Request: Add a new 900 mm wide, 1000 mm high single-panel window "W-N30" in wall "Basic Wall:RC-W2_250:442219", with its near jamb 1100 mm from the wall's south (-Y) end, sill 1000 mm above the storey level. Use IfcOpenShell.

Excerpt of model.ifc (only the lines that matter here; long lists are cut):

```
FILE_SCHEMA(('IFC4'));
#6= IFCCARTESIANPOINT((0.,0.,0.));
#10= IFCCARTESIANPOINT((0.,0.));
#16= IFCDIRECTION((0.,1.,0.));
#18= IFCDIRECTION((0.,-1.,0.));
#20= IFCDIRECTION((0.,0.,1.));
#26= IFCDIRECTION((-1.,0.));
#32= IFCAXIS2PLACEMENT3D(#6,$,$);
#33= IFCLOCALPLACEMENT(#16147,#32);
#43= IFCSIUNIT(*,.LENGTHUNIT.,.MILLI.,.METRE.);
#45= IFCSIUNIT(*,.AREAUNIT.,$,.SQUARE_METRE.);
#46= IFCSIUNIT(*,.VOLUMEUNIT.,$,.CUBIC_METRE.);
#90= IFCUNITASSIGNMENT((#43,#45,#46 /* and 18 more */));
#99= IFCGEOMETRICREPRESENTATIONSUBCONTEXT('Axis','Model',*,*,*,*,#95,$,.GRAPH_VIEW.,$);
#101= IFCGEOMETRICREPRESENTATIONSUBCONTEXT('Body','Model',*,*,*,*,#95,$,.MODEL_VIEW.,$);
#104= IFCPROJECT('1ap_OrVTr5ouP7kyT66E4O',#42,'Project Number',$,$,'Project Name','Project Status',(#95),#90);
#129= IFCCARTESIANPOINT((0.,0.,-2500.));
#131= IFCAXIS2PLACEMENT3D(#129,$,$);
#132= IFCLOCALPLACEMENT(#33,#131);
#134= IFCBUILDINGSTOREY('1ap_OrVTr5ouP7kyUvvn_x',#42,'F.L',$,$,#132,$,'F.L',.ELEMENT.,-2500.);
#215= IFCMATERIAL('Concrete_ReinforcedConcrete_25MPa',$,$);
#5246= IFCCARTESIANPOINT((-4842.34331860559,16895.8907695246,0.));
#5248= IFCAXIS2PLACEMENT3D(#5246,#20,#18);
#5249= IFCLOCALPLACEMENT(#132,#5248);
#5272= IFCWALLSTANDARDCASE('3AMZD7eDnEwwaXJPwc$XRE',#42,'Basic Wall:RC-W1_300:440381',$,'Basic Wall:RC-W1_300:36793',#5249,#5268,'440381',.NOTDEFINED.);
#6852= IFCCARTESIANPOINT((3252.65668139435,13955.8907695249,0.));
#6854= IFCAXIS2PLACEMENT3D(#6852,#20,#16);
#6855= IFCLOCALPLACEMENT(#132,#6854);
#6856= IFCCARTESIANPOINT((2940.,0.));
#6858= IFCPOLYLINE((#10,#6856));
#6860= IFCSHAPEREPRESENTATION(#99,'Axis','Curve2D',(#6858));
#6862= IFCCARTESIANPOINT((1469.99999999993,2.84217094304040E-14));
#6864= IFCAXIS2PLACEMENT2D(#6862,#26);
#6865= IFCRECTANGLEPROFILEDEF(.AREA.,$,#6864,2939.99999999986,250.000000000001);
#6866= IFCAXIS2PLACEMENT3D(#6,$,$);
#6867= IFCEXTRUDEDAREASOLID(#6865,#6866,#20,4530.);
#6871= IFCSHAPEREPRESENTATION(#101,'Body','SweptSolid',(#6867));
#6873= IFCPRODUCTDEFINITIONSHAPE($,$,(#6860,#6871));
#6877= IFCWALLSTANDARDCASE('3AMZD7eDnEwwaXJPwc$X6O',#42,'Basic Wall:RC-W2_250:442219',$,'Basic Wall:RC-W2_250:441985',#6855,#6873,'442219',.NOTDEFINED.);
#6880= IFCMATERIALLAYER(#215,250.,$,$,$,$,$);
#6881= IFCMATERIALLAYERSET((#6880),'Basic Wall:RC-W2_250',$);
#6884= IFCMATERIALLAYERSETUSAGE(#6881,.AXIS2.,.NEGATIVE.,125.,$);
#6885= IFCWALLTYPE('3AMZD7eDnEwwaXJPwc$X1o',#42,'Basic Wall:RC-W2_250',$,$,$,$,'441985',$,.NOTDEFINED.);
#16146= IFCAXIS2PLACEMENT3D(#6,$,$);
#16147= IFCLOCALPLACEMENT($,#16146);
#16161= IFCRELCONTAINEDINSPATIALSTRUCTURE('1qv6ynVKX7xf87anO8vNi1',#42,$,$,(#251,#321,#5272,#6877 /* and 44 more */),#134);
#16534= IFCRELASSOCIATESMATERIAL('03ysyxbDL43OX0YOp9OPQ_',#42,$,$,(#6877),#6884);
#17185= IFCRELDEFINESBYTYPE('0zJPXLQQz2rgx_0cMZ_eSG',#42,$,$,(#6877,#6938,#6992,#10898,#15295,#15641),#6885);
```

```python
import numpy as np
import ifcopenshell
import ifcopenshell.api.feature
import ifcopenshell.api.geometry
import ifcopenshell.api.root
import ifcopenshell.api.spatial
import ifcopenshell.geom
import ifcopenshell.util.element
import ifcopenshell.util.placement
import ifcopenshell.util.representation
import ifcopenshell.util.shape
import ifcopenshell.util.unit

model = ifcopenshell.open("model.ifc")
unit_scale = ifcopenshell.util.unit.calculate_unit_scale(model)
settings = ifcopenshell.geom.settings()


def volume(element):
    """Net volume in cubic metres, openings subtracted."""
    shape = ifcopenshell.geom.create_shape(settings, element)
    return ifcopenshell.util.shape.get_volume(shape.geometry)


wall = model.by_guid("3AMZD7eDnEwwaXJPwc$X6O")
storey = ifcopenshell.util.element.get_container(wall, ifc_class="IfcBuildingStorey")
context = ifcopenshell.util.representation.get_context(model, "Model", "Body", "MODEL_VIEW")
before = volume(wall)

width, height, from_end, sill = 0.9, 1, 1.1, 1  # metres

# The wall runs along its own X axis, and the end named is its -X end.
wall_shape = ifcopenshell.geom.create_shape(settings, wall)
x, y, z = ifcopenshell.util.shape.get_vertices(wall_shape.geometry).T
start = x.min() + from_end
face, thickness = float(y.min()), float(y.max() - y.min())
wall_matrix = ifcopenshell.util.placement.get_local_placement(wall.ObjectPlacement)
level = ifcopenshell.util.placement.get_local_placement(storey.ObjectPlacement)[2, 3]


def in_wall(x, y):
    """Placement at x, y metres in the wall's axes, at sill height."""
    matrix = wall_matrix.copy()
    matrix[:, 3] = wall_matrix @ np.array([x / unit_scale, y / unit_scale, 0.0, 1.0])
    matrix[2, 3] = level + sill / unit_scale
    return matrix


# Opening: a box that overshoots both wall faces by 50 mm.
opening = ifcopenshell.api.root.create_entity(model, ifc_class="IfcOpeningElement", predefined_type="OPENING")
box = ifcopenshell.api.geometry.add_wall_representation(
    model, context=context, length=width, height=height, thickness=thickness + 0.1
)
ifcopenshell.api.geometry.assign_representation(model, product=opening, representation=box)
ifcopenshell.api.geometry.edit_object_placement(model, product=opening, matrix=in_wall(start, face - 0.05), is_si=False)
ifcopenshell.api.feature.add_feature(model, feature=opening, element=wall)

window = ifcopenshell.api.root.create_entity(model, ifc_class="IfcWindow", name="W-N30", predefined_type="WINDOW")
window.OverallWidth, window.OverallHeight = width / unit_scale, height / unit_scale
window.PartitioningType = "SINGLE_PANEL"
body = ifcopenshell.api.geometry.add_window_representation(
    model,
    context=context,
    overall_width=window.OverallWidth,
    overall_height=window.OverallHeight,
    partition_type="SINGLE_PANEL",
)
ifcopenshell.api.geometry.assign_representation(model, product=window, representation=body)
ifcopenshell.api.spatial.assign_container(model, products=[window], relating_structure=storey)
ifcopenshell.api.feature.add_filling(model, opening=opening, element=window)

# Centre the window in the wall's thickness.
ifcopenshell.api.geometry.edit_object_placement(model, product=window, matrix=in_wall(start, face), is_si=False)
window_shape = ifcopenshell.geom.create_shape(settings, window)
depth = ifcopenshell.util.shape.get_vertices(window_shape.geometry)[:, 1]
offset = face + thickness / 2 - (depth.min() + depth.max()) / 2
ifcopenshell.api.geometry.edit_object_placement(model, product=window, matrix=in_wall(start, offset), is_si=False)

after = volume(wall)

print(f"wall volume {before:.3f} -> {after:.3f} m3")

model.write("model_rev.ifc")
```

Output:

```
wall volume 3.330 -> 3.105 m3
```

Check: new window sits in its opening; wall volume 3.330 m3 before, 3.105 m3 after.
